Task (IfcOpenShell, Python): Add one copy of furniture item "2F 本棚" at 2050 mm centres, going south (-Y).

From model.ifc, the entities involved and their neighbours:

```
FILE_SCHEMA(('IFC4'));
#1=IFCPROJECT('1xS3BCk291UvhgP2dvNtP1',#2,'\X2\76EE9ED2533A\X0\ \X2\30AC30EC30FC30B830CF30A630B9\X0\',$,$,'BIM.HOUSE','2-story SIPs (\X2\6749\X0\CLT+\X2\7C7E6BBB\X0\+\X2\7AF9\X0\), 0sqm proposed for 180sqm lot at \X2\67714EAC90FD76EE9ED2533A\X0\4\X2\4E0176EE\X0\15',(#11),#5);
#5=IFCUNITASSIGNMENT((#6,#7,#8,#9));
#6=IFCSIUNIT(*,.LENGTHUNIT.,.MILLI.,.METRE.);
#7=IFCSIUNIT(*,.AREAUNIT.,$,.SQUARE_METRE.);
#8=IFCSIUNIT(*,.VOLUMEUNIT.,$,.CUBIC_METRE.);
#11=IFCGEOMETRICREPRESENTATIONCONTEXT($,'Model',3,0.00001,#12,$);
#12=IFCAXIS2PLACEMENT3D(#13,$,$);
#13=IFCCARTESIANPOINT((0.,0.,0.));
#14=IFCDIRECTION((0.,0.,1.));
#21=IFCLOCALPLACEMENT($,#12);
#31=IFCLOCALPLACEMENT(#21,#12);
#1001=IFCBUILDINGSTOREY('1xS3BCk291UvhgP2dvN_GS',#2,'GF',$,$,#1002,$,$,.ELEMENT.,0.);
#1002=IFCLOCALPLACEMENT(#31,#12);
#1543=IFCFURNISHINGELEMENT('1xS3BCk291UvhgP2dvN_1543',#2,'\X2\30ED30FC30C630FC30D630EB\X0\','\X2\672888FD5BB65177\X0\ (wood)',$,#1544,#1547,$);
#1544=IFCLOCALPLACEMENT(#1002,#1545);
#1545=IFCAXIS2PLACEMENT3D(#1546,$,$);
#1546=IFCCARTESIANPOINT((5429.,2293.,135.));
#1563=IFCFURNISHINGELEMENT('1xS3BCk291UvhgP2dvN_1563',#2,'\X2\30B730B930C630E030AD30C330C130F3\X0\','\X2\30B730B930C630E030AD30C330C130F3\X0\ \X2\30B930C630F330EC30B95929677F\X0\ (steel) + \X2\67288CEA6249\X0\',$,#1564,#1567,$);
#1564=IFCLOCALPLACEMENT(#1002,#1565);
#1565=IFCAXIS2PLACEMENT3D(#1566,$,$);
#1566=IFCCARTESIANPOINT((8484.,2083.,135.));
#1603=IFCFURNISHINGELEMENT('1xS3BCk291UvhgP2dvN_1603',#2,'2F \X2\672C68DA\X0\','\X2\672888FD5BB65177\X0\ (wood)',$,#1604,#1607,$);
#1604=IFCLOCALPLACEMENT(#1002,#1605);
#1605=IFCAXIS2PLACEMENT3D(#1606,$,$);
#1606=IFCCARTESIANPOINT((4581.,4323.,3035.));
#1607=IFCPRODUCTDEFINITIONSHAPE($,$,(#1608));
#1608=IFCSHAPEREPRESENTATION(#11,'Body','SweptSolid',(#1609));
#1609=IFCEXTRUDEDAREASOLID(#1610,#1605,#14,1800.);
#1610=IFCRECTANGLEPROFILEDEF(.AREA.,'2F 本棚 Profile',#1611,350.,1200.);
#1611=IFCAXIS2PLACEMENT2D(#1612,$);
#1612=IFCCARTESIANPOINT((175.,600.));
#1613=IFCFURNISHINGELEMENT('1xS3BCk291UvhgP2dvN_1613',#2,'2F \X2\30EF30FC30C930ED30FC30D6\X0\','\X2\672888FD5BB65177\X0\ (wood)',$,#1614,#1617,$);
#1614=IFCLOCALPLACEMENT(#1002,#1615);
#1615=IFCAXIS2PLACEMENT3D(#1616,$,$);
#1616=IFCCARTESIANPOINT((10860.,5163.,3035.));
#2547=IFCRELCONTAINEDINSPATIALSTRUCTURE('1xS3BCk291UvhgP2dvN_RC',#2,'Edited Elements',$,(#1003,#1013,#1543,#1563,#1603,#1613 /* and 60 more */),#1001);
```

```python
import numpy as np
import ifcopenshell
import ifcopenshell.api.geometry
import ifcopenshell.api.root
import ifcopenshell.util.element
import ifcopenshell.util.placement
import ifcopenshell.util.unit

model = ifcopenshell.open("model.ifc")
unit_scale = ifcopenshell.util.unit.calculate_unit_scale(model)


def reuse_history(source, copy):
    """copy_class also copies each property set's owner history, people and application; keep the originals."""
    for rel in copy.IsDefinedBy:
        if rel.is_a("IfcRelDefinesByProperties") and (history := rel.RelatingPropertyDefinition.OwnerHistory):
            rel.RelatingPropertyDefinition.OwnerHistory = source.OwnerHistory
            ifcopenshell.util.element.remove_deep2(model, history)


source = model.by_id(1603)
base = ifcopenshell.util.placement.get_local_placement(source.ObjectPlacement)
step = np.array([0.0, -1.0, 0.0]) * 2.05 / unit_scale

for i in range(1, 2):
    copy = ifcopenshell.api.root.copy_class(model, product=source)
    copy.Representation = ifcopenshell.util.element.copy_deep(
        model, source.Representation, exclude=["IfcGeometricRepresentationContext", "IfcRepresentationMap"]
    )
    reuse_history(source, copy)
    matrix = base.copy()
    matrix[:3, 3] += i * step
    print("added at", matrix[:3, 3].round(3) + 0.0)
    ifcopenshell.api.geometry.edit_object_placement(model, product=copy, matrix=matrix, is_si=False)

model.write("model_v2.ifc")
```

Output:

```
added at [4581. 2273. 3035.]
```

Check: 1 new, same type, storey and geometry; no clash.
